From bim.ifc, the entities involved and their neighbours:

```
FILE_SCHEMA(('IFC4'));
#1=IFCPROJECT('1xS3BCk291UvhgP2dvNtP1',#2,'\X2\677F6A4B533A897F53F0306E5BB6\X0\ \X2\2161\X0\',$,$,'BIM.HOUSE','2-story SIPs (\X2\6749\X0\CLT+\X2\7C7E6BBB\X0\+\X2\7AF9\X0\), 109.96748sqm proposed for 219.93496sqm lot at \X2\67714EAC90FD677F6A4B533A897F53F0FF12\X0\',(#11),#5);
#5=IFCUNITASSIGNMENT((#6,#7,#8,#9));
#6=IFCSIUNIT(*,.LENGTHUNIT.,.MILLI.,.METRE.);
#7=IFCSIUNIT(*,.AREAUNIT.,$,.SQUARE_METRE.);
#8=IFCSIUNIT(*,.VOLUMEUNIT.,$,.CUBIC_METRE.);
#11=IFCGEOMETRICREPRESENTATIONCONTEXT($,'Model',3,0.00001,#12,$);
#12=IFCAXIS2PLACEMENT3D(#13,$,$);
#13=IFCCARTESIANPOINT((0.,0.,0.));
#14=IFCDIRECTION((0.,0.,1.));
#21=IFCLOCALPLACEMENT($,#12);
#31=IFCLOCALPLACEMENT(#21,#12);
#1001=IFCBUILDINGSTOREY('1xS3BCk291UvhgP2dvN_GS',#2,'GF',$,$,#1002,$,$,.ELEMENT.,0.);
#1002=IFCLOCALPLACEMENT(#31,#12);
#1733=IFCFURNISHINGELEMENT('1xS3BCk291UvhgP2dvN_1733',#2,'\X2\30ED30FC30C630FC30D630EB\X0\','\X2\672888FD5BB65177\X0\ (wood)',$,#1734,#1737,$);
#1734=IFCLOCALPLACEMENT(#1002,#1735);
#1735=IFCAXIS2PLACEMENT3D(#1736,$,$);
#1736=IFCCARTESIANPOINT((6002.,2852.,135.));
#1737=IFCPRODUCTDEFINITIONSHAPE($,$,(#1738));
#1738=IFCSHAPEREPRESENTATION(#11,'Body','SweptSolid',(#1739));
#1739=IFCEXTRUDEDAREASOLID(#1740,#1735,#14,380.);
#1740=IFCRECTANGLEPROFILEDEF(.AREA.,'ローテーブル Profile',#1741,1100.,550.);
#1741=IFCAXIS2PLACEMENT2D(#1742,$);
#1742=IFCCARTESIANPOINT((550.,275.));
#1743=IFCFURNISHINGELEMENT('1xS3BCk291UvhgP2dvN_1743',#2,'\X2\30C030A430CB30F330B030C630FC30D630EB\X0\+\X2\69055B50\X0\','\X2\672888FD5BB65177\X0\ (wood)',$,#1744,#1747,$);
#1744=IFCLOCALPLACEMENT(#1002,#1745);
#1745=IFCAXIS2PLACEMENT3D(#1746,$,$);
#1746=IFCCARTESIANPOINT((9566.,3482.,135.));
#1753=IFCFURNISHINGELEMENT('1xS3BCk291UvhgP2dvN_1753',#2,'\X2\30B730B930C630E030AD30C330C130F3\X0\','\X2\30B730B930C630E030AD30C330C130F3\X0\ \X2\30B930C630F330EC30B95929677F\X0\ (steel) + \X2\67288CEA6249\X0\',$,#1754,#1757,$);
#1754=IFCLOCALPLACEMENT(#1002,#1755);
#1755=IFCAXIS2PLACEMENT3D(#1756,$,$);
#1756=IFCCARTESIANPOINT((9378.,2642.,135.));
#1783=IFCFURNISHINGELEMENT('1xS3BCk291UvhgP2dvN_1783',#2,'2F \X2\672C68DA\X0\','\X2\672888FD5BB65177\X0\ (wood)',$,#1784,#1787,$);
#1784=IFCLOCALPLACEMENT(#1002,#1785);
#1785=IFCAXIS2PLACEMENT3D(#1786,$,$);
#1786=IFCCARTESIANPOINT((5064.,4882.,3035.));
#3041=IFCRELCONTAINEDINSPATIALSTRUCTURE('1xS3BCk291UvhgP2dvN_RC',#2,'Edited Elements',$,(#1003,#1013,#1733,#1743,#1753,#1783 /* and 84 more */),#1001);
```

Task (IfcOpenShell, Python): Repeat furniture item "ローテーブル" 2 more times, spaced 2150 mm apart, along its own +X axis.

```python
import ifcopenshell
import ifcopenshell.api.geometry
import ifcopenshell.api.root
import ifcopenshell.util.element
import ifcopenshell.util.placement
import ifcopenshell.util.unit

model = ifcopenshell.open("bim.ifc")
unit_scale = ifcopenshell.util.unit.calculate_unit_scale(model)


def reuse_history(source, copy):
    """copy_class also copies each property set's owner history, people and application; keep the originals."""
    for rel in copy.IsDefinedBy:
        if rel.is_a("IfcRelDefinesByProperties") and (history := rel.RelatingPropertyDefinition.OwnerHistory):
            rel.RelatingPropertyDefinition.OwnerHistory = source.OwnerHistory
            ifcopenshell.util.element.remove_deep2(model, history)


source = model.by_guid("1xS3BCk291UvhgP2dvN_1733")
base = ifcopenshell.util.placement.get_local_placement(source.ObjectPlacement)
step = base[:3, 0] * 2.15 / unit_scale

for i in range(1, 3):
    copy = ifcopenshell.api.root.copy_class(model, product=source)
    copy.Representation = ifcopenshell.util.element.copy_deep(
        model, source.Representation, exclude=["IfcGeometricRepresentationContext", "IfcRepresentationMap"]
    )
    reuse_history(source, copy)
    matrix = base.copy()
    matrix[:3, 3] += i * step
    print("added at", matrix[:3, 3].round(3) + 0.0)
    ifcopenshell.api.geometry.edit_object_placement(model, product=copy, matrix=matrix, is_si=False)

model.write("bim_edited.ifc")
```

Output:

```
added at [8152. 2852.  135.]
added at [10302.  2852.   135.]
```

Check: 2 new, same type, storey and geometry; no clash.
